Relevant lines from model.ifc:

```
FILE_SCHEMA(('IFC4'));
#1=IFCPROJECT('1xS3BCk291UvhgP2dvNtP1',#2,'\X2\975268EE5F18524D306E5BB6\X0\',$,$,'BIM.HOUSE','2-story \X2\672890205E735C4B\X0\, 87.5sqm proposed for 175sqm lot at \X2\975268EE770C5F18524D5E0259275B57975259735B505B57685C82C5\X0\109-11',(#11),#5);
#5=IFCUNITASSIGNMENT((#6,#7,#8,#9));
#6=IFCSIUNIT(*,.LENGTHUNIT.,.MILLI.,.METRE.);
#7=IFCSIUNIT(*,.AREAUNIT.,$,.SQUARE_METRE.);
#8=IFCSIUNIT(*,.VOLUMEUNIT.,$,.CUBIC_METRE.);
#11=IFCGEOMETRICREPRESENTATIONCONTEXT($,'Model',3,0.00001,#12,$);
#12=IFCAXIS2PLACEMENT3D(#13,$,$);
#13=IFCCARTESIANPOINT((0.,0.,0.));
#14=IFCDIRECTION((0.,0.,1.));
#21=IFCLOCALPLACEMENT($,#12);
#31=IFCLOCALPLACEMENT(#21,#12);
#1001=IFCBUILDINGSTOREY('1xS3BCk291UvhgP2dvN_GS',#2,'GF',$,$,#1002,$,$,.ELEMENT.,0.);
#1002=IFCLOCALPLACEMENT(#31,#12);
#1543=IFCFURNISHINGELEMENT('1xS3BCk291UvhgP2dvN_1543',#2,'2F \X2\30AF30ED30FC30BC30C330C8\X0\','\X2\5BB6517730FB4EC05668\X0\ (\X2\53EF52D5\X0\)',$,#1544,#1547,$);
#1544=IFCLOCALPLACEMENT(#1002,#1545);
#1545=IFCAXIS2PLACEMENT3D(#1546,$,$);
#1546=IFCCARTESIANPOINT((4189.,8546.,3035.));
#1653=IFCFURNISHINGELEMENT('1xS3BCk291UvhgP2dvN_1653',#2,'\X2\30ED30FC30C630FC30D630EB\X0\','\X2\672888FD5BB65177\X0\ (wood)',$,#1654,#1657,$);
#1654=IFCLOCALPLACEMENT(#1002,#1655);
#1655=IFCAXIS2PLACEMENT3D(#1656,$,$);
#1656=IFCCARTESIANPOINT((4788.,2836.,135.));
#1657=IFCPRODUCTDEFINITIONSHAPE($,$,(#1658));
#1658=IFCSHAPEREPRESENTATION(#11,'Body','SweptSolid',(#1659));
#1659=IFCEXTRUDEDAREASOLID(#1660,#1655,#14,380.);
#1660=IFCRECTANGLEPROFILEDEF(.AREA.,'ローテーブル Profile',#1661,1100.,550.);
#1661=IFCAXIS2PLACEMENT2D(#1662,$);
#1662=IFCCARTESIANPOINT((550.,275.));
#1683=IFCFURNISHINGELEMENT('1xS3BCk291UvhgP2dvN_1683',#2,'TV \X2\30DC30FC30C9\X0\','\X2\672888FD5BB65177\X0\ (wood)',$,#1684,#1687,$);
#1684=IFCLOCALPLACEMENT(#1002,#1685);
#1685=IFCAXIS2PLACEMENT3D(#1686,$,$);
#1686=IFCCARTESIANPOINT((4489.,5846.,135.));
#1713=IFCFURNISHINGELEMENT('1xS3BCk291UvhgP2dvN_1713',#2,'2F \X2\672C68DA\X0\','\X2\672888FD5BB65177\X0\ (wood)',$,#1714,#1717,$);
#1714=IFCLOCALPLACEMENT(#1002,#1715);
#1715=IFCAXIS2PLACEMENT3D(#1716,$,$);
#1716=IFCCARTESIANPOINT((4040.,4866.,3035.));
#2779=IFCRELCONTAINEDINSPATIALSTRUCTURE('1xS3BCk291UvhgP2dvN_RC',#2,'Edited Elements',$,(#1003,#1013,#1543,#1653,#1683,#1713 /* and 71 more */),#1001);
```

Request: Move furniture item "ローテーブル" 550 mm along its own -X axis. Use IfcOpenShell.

```python
import ifcopenshell
import ifcopenshell.api.geometry
import ifcopenshell.util.placement
import ifcopenshell.util.unit

model = ifcopenshell.open("model.ifc")
unit_scale = ifcopenshell.util.unit.calculate_unit_scale(model)

item = model.by_guid("1xS3BCk291UvhgP2dvN_1653")
matrix = ifcopenshell.util.placement.get_local_placement(item.ObjectPlacement)
matrix[:3, 3] -= matrix[:3, 0] * 0.55 / unit_scale
ifcopenshell.api.geometry.edit_object_placement(model, product=item, matrix=matrix, is_si=False)

print(ifcopenshell.util.placement.get_local_placement(item.ObjectPlacement).round(3) + 0.0)

model.write("model_updated.ifc")
```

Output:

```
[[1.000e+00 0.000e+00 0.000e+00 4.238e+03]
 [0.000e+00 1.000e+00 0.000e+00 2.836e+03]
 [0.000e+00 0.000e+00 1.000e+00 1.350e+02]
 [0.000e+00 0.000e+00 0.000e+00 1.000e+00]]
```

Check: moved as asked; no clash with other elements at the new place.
